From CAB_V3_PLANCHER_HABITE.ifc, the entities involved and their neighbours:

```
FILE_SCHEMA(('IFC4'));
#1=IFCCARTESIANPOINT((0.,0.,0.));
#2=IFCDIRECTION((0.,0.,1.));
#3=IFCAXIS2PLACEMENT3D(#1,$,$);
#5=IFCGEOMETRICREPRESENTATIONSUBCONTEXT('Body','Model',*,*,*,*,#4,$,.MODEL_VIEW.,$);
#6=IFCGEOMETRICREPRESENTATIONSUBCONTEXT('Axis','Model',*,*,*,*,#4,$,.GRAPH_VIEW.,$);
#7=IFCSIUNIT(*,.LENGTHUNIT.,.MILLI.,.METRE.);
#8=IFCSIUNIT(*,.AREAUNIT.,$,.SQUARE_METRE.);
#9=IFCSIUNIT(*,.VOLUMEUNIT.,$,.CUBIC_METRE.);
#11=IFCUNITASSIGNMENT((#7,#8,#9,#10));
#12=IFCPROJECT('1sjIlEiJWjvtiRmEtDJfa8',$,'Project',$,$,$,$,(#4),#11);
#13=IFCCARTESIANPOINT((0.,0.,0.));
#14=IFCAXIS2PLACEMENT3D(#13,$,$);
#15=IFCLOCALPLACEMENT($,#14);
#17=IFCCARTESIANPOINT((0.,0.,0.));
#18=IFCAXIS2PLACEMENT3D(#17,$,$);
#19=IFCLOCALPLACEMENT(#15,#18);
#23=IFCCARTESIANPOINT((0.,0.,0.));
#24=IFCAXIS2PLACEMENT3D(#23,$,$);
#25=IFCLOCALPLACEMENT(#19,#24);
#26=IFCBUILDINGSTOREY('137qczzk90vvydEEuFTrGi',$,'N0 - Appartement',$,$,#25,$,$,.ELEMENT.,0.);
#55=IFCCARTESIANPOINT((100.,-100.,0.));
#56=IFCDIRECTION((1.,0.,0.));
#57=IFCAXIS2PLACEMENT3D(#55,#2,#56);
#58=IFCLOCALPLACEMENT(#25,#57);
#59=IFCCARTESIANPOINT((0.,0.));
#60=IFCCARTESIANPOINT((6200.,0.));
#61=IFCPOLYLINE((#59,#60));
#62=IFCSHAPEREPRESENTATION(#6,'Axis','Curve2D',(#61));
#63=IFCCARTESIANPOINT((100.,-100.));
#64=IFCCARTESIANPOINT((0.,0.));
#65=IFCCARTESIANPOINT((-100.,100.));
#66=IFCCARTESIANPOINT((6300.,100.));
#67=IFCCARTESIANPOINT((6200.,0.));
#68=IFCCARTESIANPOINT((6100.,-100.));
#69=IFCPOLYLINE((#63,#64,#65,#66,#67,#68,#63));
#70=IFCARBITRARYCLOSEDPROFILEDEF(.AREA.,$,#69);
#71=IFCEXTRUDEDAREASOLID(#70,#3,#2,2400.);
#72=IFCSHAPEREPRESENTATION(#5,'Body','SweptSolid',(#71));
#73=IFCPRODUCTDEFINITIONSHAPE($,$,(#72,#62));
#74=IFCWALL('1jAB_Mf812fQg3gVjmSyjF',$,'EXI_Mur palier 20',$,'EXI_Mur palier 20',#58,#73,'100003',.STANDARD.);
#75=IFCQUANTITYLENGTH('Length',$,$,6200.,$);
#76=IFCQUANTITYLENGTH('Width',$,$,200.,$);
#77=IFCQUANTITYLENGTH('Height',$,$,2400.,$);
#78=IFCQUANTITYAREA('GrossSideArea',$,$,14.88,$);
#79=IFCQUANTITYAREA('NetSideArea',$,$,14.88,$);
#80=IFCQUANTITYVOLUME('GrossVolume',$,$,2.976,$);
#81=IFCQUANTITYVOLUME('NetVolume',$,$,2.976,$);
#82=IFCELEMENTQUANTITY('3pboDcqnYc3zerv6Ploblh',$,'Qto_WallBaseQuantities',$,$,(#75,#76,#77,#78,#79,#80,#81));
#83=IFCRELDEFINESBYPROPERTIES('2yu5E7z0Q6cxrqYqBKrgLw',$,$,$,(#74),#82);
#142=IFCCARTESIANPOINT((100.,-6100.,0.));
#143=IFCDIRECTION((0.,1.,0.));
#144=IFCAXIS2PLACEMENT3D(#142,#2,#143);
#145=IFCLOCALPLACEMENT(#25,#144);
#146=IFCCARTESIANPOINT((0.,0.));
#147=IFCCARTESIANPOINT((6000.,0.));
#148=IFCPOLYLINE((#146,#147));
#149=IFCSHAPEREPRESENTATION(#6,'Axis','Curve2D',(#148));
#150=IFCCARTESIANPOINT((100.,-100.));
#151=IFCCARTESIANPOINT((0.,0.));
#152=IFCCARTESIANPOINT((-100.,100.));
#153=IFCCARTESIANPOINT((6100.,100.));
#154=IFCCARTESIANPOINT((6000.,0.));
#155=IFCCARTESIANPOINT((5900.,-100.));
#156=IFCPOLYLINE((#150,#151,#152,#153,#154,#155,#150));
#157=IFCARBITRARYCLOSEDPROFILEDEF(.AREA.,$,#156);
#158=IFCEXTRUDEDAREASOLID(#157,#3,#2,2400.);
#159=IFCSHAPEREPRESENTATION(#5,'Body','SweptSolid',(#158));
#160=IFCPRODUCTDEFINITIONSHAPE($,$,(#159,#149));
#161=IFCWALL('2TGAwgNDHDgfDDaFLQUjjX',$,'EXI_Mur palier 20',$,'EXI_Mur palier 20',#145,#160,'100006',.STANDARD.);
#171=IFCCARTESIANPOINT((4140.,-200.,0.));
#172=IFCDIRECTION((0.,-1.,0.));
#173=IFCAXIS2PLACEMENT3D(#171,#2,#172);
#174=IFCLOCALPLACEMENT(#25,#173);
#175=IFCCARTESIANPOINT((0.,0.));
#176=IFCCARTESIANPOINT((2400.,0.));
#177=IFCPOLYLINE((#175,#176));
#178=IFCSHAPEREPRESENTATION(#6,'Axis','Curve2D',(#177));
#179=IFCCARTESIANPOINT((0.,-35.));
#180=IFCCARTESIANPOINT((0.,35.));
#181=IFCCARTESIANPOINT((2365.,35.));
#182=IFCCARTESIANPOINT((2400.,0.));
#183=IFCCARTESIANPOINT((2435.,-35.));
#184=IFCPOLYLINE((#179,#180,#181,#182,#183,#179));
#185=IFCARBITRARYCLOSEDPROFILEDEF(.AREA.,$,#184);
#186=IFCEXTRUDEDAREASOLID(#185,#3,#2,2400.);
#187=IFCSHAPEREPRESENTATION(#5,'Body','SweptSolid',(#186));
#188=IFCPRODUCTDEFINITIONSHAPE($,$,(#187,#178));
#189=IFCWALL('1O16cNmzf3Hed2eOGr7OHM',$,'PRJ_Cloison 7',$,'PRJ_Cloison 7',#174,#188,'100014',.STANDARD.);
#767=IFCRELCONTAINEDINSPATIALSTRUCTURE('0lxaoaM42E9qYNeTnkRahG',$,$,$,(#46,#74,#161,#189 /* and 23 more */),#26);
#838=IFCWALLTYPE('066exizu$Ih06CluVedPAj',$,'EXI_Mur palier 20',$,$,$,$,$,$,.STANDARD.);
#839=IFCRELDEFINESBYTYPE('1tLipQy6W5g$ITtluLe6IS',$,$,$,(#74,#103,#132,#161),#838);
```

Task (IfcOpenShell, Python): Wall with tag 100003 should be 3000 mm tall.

```python
import ifcopenshell
import ifcopenshell.api.pset
import ifcopenshell.geom
import ifcopenshell.util.element
import ifcopenshell.util.representation
import ifcopenshell.util.shape
import ifcopenshell.util.unit

model = ifcopenshell.open("CAB_V3_PLANCHER_HABITE.ifc")
unit_scale = ifcopenshell.util.unit.calculate_unit_scale(model)
area_scale = ifcopenshell.util.unit.calculate_unit_scale(model, "AREAUNIT")
volume_scale = ifcopenshell.util.unit.calculate_unit_scale(model, "VOLUMEUNIT")
settings = ifcopenshell.geom.settings()


def volume(element):
    """Net volume in cubic metres, openings subtracted."""
    shape = ifcopenshell.geom.create_shape(settings, element)
    return ifcopenshell.util.shape.get_volume(shape.geometry)


wall = model.by_guid("1jAB_Mf812fQg3gVjmSyjF")
before = volume(wall)

body = ifcopenshell.util.representation.get_representation(wall, "Model", "Body")
solid = body.Items[0]
old_height = solid.Depth
solid.Depth = 3 / unit_scale
after = volume(wall)
thickness = 0.2  # wall thickness in metres

# Update the stored height, areas and volumes.
qto = model.by_id(ifcopenshell.util.element.get_pset(wall, "Qto_WallBaseQuantities", should_inherit=False)["id"])
ifcopenshell.api.pset.edit_qto(model, qto=qto, properties={
    "Height": solid.Depth,
    "GrossSideArea": ifcopenshell.util.element.get_pset(wall, "Qto_WallBaseQuantities", "GrossSideArea") * solid.Depth / old_height,
    "NetSideArea": after / thickness / area_scale,
    "GrossVolume": ifcopenshell.util.element.get_pset(wall, "Qto_WallBaseQuantities", "GrossVolume") * solid.Depth / old_height,
    "NetVolume": after / volume_scale,
})

print(f"height {old_height:g} -> {solid.Depth:g}, volume {before:.3f} -> {after:.3f} m3")

model.write("CAB_V3_PLANCHER_HABITE_edited.ifc")
```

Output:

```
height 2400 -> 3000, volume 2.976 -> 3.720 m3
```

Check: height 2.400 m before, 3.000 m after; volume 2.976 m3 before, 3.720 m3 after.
